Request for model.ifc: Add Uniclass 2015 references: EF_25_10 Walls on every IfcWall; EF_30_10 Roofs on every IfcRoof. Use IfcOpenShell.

First a look at what the model holds.

```python
import ifcopenshell

model = ifcopenshell.open("model.ifc")
print(model.schema)
print("classifications:", [c.Name for c in model.by_type("IfcClassification")])
for ifc_class in ("IfcDoor", "IfcRoof", "IfcStair", "IfcWall", "IfcWindow"):
    print(ifc_class, len(model.by_type(ifc_class)))
```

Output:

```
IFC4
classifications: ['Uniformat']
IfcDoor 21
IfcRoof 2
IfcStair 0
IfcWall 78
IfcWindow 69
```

```python
import ifcopenshell
import ifcopenshell.api.classification

model = ifcopenshell.open("model.ifc")

system = ifcopenshell.api.classification.add_classification(model, classification="Uniclass 2015")

codes = {
    "IfcWall": ("EF_25_10", "Walls"),
    "IfcRoof": ("EF_30_10", "Roofs"),
}
for ifc_class, (code, name) in codes.items():
    products = model.by_type(ifc_class)
    ifcopenshell.api.classification.add_reference(
        model, products=products, classification=system, identification=code, name=name
    )
    print(code, len(products))

model.write("model-out.ifc")
```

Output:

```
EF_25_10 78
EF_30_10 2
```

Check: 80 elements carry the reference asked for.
